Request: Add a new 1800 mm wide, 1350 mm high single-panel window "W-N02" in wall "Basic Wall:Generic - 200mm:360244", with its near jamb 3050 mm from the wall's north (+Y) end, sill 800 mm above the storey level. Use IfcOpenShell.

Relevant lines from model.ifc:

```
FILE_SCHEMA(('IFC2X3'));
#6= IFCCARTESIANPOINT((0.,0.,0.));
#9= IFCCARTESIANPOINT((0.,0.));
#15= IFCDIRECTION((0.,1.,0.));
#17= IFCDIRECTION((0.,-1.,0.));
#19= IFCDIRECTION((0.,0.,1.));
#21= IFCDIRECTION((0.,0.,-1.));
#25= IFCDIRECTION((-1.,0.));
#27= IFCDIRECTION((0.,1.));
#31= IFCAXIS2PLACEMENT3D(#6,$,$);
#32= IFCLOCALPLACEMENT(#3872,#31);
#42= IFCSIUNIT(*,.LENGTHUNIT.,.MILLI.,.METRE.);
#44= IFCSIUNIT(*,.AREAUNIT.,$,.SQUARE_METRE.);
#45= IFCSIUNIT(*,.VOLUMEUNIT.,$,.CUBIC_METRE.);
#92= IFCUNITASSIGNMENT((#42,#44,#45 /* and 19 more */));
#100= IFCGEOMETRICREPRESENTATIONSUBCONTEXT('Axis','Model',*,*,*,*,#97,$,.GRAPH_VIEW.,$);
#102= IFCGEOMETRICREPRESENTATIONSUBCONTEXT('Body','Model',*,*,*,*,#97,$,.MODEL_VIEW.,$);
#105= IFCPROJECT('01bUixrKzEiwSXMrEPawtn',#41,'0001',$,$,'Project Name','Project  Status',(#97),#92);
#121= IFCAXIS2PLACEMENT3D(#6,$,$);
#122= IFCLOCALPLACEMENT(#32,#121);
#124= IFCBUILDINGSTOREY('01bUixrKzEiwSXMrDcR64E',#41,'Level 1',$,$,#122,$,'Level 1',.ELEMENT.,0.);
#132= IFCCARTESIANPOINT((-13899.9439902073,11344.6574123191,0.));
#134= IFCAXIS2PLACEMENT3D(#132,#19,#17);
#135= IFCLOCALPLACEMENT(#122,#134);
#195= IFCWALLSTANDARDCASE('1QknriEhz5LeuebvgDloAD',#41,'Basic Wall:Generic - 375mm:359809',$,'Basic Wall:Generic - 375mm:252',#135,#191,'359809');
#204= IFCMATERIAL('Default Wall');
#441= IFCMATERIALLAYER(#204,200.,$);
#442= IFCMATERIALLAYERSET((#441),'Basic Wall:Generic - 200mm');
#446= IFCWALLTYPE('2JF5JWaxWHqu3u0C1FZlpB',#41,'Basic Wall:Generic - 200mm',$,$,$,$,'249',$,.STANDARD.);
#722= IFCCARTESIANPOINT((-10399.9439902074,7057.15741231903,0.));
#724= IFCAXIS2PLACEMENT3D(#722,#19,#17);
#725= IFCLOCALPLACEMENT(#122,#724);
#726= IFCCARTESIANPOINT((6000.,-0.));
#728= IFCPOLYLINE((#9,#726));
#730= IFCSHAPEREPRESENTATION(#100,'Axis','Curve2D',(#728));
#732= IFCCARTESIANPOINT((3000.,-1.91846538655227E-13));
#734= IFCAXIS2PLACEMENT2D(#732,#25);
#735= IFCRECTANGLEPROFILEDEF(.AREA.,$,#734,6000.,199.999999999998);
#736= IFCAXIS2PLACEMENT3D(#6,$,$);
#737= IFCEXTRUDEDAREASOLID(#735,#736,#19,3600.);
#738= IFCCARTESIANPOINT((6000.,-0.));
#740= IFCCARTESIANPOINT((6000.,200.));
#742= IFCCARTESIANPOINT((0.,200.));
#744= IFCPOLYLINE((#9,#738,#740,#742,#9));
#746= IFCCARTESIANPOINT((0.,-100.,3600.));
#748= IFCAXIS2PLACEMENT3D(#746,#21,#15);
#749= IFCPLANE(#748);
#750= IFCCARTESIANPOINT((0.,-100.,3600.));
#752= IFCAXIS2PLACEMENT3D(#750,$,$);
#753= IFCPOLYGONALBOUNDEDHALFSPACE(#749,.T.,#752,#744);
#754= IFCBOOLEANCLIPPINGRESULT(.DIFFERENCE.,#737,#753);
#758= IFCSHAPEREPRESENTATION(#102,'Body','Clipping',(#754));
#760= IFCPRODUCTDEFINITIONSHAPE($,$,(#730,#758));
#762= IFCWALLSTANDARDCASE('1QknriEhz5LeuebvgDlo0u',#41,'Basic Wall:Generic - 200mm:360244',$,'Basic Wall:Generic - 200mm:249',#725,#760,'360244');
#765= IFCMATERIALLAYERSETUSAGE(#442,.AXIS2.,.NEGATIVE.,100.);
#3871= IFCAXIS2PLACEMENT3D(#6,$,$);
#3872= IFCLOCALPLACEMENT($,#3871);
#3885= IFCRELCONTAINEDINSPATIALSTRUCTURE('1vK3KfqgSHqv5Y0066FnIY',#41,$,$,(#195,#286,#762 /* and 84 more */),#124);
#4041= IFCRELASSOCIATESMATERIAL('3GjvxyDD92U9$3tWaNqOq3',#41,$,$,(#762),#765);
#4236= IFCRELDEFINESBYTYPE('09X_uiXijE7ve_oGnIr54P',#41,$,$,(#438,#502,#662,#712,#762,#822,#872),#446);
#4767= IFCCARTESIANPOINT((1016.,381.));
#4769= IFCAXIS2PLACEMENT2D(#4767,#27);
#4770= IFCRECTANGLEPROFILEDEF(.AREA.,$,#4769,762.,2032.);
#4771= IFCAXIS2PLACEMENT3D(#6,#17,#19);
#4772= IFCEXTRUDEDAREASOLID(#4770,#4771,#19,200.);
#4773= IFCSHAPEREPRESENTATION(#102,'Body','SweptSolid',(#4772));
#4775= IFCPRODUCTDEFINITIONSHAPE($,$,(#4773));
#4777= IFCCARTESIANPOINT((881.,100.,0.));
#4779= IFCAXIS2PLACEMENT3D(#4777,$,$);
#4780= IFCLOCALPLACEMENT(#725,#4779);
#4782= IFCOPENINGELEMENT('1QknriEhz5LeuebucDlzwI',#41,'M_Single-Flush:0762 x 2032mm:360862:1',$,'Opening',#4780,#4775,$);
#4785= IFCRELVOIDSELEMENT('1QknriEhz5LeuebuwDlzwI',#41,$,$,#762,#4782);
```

```python
import numpy as np
import ifcopenshell
import ifcopenshell.api.feature
import ifcopenshell.api.geometry
import ifcopenshell.api.root
import ifcopenshell.api.spatial
import ifcopenshell.api.type
import ifcopenshell.geom
import ifcopenshell.util.element
import ifcopenshell.util.placement
import ifcopenshell.util.representation
import ifcopenshell.util.shape
import ifcopenshell.util.unit

model = ifcopenshell.open("model.ifc")
unit_scale = ifcopenshell.util.unit.calculate_unit_scale(model)
settings = ifcopenshell.geom.settings()


def volume(element):
    """Net volume in cubic metres, openings subtracted."""
    shape = ifcopenshell.geom.create_shape(settings, element)
    return ifcopenshell.util.shape.get_volume(shape.geometry)


wall = model.by_id(762)
storey = ifcopenshell.util.element.get_container(wall, ifc_class="IfcBuildingStorey")
context = ifcopenshell.util.representation.get_context(model, "Model", "Body", "MODEL_VIEW")
before = volume(wall)

width, height, from_end, sill = 1.8, 1.35, 3.05, 0.8  # metres

# The wall runs along its own X axis, and the end named is its -X end.
wall_shape = ifcopenshell.geom.create_shape(settings, wall)
x, y, z = ifcopenshell.util.shape.get_vertices(wall_shape.geometry).T
start = x.min() + from_end
face, thickness = float(y.min()), float(y.max() - y.min())
wall_matrix = ifcopenshell.util.placement.get_local_placement(wall.ObjectPlacement)
level = ifcopenshell.util.placement.get_local_placement(storey.ObjectPlacement)[2, 3]


def in_wall(x, y):
    """Placement at x, y metres in the wall's axes, at sill height."""
    matrix = wall_matrix.copy()
    matrix[:, 3] = wall_matrix @ np.array([x / unit_scale, y / unit_scale, 0.0, 1.0])
    matrix[2, 3] = level + sill / unit_scale
    return matrix


# Opening: a box that overshoots both wall faces by 50 mm.
opening = ifcopenshell.api.root.create_entity(model, ifc_class="IfcOpeningElement")
box = ifcopenshell.api.geometry.add_wall_representation(
    model, context=context, length=width, height=height, thickness=thickness + 0.1
)
ifcopenshell.api.geometry.assign_representation(model, product=opening, representation=box)
ifcopenshell.api.geometry.edit_object_placement(model, product=opening, matrix=in_wall(start, face - 0.05), is_si=False)
ifcopenshell.api.feature.add_feature(model, feature=opening, element=wall)

window = ifcopenshell.api.root.create_entity(model, ifc_class="IfcWindow", name="W-N02")
window.OverallWidth, window.OverallHeight = width / unit_scale, height / unit_scale
body = ifcopenshell.api.geometry.add_window_representation(
    model,
    context=context,
    overall_width=window.OverallWidth,
    overall_height=window.OverallHeight,
    partition_type="SINGLE_PANEL",
)
ifcopenshell.api.geometry.assign_representation(model, product=window, representation=body)
ifcopenshell.api.spatial.assign_container(model, products=[window], relating_structure=storey)
fills = ifcopenshell.api.feature.add_filling(model, opening=opening, element=window)
fills.OwnerHistory = window.OwnerHistory  # required in IFC2X3

# IFC2X3 keeps the operation on the window style.
style = ifcopenshell.api.root.create_entity(model, ifc_class="IfcWindowStyle", name="W-N02")
style.OperationType, style.ConstructionType = "SINGLE_PANEL", "NOTDEFINED"
style.ParameterTakesPrecedence = style.Sizeable = False
ifcopenshell.api.type.assign_type(model, related_objects=[window], relating_type=style)

# Centre the window in the wall's thickness.
ifcopenshell.api.geometry.edit_object_placement(model, product=window, matrix=in_wall(start, face), is_si=False)
window_shape = ifcopenshell.geom.create_shape(settings, window)
depth = ifcopenshell.util.shape.get_vertices(window_shape.geometry)[:, 1]
offset = face + thickness / 2 - (depth.min() + depth.max()) / 2
ifcopenshell.api.geometry.edit_object_placement(model, product=window, matrix=in_wall(start, offset), is_si=False)

after = volume(wall)

print(f"wall volume {before:.3f} -> {after:.3f} m3")

model.write("model_v2.ifc")
```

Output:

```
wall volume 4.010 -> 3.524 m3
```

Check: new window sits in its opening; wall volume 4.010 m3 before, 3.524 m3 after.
